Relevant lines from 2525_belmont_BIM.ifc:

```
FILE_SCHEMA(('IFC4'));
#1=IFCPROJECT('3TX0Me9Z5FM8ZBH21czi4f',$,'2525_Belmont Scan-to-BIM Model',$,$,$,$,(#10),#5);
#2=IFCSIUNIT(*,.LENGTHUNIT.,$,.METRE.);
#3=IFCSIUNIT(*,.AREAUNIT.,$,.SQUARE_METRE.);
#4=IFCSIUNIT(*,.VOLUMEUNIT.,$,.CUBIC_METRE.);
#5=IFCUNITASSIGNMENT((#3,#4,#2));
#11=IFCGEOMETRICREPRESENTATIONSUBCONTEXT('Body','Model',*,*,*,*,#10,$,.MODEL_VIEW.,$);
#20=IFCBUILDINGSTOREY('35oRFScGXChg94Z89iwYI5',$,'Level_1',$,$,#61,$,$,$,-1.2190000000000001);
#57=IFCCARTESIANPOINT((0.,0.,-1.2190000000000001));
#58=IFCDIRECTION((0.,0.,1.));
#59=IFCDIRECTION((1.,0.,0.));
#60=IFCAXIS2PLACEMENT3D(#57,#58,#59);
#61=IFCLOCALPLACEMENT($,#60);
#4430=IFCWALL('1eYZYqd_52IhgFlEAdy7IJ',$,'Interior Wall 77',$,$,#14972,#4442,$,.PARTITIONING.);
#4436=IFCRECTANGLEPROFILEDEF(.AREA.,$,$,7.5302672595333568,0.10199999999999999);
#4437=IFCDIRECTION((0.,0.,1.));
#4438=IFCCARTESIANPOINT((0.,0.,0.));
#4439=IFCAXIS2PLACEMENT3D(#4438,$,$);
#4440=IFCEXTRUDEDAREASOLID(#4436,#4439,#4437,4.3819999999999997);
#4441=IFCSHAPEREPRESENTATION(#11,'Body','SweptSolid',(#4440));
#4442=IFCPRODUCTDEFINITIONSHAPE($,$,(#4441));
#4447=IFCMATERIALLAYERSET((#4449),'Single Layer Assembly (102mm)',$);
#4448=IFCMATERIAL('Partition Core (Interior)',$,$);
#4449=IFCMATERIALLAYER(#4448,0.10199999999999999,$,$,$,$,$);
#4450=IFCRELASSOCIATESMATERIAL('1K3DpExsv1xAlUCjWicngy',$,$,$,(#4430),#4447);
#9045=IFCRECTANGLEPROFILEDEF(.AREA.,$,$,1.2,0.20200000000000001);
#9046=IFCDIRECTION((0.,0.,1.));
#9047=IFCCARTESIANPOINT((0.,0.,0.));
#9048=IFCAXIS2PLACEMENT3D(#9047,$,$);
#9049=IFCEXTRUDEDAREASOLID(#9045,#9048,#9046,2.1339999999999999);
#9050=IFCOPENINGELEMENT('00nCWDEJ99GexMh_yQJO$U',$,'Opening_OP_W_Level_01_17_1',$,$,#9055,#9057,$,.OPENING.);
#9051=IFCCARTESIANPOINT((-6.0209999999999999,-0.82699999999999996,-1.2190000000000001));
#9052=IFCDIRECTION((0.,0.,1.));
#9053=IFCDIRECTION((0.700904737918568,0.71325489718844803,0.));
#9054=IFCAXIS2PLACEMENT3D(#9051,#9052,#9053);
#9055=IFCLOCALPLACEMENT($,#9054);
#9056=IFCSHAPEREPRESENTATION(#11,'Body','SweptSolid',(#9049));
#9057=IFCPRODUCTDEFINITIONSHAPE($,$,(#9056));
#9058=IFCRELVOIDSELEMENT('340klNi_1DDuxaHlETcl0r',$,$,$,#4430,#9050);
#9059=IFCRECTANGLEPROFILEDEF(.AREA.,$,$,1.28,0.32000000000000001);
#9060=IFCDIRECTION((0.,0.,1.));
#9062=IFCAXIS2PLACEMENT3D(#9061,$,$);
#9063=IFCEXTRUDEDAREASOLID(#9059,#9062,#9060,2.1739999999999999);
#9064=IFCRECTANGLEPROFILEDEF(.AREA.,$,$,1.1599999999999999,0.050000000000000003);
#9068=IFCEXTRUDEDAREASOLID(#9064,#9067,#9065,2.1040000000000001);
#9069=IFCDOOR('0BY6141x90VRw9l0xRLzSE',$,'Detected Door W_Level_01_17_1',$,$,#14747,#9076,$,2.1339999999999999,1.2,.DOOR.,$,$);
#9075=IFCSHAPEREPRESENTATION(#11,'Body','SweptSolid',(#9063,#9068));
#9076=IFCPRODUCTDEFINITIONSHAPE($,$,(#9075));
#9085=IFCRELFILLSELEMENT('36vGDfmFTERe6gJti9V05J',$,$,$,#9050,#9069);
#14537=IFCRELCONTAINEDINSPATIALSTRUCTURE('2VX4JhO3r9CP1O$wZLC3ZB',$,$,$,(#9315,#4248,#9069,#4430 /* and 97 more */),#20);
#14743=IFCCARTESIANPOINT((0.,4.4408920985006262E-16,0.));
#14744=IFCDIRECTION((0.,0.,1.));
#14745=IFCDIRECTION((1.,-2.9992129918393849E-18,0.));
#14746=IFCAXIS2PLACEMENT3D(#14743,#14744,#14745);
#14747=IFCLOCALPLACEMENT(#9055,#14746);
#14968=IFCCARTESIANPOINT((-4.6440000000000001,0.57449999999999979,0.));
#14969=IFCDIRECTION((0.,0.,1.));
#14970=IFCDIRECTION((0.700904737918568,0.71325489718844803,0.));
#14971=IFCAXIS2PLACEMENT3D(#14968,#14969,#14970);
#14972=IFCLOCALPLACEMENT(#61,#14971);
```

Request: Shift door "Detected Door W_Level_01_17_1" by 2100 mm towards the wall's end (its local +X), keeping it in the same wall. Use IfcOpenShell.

```python
import ifcopenshell
import ifcopenshell.api.geometry
import ifcopenshell.util.placement
import ifcopenshell.util.unit

model = ifcopenshell.open("2525_belmont_BIM.ifc")
unit_scale = ifcopenshell.util.unit.calculate_unit_scale(model)

door = model.by_guid("0BY6141x90VRw9l0xRLzSE")
opening = door.FillsVoids[0].RelatingOpeningElement
wall = opening.VoidsElements[0].RelatingBuildingElement

wall_matrix = ifcopenshell.util.placement.get_local_placement(wall.ObjectPlacement)
shift = wall_matrix[:3, 0] * 2.1 / unit_scale
before = ifcopenshell.util.placement.get_local_placement(door.ObjectPlacement)[:3, 3].copy()

# The door is placed relative to its opening, so it follows when the opening moves.
matrix = ifcopenshell.util.placement.get_local_placement(opening.ObjectPlacement)
matrix[:3, 3] += shift
ifcopenshell.api.geometry.edit_object_placement(
    model, product=opening, matrix=matrix, is_si=False, should_transform_children=True
)

after = ifcopenshell.util.placement.get_local_placement(door.ObjectPlacement)[:3, 3]
print("door moved by", (after - before).round(3) + 0.0)

model.write("2525_belmont_BIM_updated.ifc")
```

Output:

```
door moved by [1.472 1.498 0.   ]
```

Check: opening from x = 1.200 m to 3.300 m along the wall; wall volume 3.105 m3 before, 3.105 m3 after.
